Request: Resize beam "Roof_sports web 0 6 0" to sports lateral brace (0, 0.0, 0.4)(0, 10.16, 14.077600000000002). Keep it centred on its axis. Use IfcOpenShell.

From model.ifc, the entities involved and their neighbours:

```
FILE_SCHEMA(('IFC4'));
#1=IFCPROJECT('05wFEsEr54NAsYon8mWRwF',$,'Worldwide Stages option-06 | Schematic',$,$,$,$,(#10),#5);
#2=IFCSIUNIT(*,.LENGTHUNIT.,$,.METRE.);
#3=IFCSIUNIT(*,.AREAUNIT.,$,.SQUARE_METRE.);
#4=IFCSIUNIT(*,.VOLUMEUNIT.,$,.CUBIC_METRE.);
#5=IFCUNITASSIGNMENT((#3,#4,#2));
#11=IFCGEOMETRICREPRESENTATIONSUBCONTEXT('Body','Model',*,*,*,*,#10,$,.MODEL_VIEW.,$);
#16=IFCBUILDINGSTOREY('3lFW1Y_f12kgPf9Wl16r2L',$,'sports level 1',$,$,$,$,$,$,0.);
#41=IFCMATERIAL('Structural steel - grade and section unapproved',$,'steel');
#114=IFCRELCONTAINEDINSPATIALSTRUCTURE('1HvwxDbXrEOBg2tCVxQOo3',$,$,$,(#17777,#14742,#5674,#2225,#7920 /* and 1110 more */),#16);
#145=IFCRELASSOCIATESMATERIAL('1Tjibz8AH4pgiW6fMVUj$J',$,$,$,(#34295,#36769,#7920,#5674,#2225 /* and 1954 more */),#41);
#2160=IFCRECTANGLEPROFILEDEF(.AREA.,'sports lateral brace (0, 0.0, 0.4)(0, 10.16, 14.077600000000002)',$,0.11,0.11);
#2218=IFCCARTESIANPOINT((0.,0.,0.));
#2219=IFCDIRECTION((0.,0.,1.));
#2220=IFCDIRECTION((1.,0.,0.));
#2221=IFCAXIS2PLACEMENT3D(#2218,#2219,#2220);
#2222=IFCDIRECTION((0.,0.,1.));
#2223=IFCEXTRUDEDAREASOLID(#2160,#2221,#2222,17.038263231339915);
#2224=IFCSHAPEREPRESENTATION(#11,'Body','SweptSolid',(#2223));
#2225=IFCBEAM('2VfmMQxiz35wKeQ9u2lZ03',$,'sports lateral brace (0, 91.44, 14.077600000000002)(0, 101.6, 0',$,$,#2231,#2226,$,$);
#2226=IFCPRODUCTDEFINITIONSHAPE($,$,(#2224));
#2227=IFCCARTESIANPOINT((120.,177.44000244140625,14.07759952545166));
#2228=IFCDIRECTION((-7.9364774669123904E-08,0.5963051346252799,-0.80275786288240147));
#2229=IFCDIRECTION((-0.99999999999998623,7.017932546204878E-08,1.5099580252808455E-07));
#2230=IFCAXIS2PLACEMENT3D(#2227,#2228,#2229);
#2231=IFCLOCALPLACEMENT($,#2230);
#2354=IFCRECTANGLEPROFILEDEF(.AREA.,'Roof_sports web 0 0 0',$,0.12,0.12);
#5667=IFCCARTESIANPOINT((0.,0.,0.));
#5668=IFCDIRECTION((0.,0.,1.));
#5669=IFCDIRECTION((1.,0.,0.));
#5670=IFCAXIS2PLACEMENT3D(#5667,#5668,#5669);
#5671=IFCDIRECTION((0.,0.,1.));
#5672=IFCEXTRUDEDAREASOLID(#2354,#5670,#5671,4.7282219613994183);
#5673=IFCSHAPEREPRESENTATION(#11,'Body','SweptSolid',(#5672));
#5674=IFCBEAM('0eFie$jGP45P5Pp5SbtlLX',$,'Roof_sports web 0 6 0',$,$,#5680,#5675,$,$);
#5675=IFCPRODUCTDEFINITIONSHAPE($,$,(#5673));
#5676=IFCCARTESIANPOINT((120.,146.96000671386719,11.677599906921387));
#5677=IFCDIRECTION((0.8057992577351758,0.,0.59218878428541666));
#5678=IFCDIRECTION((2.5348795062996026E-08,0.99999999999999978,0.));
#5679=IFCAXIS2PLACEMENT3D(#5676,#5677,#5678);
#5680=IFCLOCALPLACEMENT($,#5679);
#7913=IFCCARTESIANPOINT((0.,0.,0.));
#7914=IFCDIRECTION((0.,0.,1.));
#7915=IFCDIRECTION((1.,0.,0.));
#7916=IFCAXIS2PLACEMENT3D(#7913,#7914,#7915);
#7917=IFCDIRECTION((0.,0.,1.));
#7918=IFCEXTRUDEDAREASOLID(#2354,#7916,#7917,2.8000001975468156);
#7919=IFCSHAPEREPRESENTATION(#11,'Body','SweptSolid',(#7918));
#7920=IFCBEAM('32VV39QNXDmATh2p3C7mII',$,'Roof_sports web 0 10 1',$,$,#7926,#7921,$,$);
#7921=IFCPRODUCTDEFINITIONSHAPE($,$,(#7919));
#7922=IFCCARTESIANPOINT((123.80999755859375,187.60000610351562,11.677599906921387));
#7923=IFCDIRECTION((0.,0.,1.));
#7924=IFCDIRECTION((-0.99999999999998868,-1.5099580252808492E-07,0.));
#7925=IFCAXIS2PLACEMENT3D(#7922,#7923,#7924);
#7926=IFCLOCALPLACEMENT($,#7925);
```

```python
import ifcopenshell
import ifcopenshell.util.element
import ifcopenshell.util.representation

model = ifcopenshell.open("model.ifc")

member = model.by_id(5674)
source = next(p for p in model.by_type("IfcRectangleProfileDef") if p.ProfileName == "sports lateral brace (0, 0.0, 0.4)(0, 10.16, 14.077600000000002)")

body = ifcopenshell.util.representation.get_representation(member, "Model", "Body")
solid = body.Items[0]
old_profile = solid.SweptArea

# Copy the section's sizes but keep this member's own profile position.
profile = ifcopenshell.util.element.copy(model, source)
profile.Position = old_profile.Position
solid.SweptArea = profile
if not model.get_total_inverses(old_profile):
    ifcopenshell.util.element.remove_deep2(model, old_profile)

print(solid.SweptArea)

model.write("model_edited.ifc")
```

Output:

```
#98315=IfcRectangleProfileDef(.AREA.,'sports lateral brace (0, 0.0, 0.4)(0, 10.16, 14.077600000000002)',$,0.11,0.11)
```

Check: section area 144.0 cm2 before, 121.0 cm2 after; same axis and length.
